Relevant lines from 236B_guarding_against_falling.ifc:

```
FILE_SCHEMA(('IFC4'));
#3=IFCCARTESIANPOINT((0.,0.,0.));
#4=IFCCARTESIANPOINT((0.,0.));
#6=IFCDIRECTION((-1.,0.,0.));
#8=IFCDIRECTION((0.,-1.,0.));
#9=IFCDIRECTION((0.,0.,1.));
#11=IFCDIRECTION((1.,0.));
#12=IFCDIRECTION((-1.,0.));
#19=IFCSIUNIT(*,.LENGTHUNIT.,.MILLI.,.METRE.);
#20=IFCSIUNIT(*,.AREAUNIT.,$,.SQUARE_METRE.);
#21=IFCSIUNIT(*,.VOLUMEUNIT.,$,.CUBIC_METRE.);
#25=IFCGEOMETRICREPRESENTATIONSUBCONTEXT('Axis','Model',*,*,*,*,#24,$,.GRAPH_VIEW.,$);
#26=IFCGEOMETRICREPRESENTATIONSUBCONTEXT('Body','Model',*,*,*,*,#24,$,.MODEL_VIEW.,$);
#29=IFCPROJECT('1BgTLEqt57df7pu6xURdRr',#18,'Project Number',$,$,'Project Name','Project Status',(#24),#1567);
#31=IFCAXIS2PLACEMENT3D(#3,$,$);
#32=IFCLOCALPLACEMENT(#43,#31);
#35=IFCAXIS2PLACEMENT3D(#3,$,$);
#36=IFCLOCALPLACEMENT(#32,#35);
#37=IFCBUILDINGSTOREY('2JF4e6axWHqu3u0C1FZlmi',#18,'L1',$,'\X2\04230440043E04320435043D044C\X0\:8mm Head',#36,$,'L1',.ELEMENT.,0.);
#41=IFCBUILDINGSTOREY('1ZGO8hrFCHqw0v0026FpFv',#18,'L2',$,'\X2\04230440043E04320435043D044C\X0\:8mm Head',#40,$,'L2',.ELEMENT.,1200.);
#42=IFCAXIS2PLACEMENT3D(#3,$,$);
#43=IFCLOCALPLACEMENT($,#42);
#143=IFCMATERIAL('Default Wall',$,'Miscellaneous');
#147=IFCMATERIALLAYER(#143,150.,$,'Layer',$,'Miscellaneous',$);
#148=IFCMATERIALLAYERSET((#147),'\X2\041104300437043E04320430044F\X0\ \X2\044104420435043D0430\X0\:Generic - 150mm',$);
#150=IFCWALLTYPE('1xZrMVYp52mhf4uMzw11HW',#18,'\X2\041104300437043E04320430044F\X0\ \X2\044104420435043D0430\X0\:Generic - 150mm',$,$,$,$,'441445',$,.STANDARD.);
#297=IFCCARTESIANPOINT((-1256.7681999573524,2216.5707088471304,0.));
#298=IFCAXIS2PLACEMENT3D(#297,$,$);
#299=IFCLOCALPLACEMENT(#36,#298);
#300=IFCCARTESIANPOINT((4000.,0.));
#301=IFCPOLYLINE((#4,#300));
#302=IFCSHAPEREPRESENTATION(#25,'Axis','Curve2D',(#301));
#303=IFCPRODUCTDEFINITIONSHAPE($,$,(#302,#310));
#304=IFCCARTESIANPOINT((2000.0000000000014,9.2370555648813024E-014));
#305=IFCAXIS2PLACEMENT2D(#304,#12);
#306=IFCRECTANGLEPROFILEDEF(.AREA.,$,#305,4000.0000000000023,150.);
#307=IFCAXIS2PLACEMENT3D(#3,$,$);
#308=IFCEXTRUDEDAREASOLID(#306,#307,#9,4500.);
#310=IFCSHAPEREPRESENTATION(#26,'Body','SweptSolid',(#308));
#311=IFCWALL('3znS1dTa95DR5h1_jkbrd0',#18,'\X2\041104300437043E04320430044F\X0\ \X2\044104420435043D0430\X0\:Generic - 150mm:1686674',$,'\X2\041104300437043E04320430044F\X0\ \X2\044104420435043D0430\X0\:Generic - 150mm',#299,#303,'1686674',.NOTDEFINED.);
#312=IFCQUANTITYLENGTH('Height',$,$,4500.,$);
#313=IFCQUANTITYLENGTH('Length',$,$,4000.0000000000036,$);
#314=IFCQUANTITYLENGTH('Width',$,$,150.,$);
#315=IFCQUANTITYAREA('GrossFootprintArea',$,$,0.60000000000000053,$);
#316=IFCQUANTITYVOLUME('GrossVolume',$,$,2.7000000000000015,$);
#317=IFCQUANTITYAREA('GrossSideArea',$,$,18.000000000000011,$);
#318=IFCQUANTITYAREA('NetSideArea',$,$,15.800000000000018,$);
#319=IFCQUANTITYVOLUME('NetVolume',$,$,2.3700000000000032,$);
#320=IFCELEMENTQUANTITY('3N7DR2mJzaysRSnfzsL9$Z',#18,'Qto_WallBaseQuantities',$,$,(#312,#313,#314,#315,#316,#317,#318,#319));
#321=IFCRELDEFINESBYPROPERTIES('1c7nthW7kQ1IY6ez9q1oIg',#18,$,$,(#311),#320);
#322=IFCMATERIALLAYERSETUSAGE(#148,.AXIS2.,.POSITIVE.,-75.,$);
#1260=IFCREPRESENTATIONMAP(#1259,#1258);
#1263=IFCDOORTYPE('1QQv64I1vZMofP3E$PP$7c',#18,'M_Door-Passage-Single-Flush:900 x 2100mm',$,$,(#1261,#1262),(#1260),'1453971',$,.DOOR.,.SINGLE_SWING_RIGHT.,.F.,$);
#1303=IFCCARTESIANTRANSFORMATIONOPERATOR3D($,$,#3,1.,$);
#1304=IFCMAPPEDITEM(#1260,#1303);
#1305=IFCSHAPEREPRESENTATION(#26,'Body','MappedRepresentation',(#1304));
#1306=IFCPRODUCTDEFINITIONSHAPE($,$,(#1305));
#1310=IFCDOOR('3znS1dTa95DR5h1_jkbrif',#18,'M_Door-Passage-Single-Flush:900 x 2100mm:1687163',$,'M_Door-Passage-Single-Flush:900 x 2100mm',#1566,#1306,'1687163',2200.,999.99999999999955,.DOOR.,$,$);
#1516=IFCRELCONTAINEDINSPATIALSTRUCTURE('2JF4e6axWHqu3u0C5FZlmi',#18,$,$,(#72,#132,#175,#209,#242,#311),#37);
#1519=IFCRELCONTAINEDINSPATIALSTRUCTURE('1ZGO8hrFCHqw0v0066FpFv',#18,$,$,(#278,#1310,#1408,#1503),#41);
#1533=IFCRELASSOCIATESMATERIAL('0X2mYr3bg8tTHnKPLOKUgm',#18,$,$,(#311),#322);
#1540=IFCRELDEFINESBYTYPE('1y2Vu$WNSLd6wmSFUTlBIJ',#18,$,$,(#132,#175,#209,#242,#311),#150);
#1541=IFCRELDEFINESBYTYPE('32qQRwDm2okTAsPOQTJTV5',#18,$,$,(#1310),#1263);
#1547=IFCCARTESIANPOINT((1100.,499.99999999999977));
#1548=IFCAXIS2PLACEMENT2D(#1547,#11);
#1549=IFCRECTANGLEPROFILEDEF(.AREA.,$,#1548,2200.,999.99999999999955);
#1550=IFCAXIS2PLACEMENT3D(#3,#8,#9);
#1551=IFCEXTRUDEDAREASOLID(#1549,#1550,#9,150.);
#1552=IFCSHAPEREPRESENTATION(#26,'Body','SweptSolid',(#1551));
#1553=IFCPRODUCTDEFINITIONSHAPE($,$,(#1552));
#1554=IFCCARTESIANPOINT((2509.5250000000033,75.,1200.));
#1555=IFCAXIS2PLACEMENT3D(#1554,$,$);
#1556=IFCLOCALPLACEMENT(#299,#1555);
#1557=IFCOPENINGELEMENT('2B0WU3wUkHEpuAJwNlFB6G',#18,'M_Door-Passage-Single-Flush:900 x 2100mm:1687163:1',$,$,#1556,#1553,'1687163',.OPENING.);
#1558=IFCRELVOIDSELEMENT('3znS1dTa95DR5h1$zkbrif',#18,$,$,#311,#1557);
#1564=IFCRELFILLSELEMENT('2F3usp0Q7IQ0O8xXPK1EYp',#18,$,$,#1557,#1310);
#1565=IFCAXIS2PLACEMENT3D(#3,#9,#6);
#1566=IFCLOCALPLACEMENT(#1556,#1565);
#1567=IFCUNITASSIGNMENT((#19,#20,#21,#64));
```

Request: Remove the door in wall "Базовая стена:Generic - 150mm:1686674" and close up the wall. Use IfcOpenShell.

```python
import ifcopenshell
import ifcopenshell.api.feature
import ifcopenshell.api.pset
import ifcopenshell.api.root
import ifcopenshell.geom
import ifcopenshell.util.element
import ifcopenshell.util.shape
import ifcopenshell.util.unit

model = ifcopenshell.open("236B_guarding_against_falling.ifc")
area_scale = ifcopenshell.util.unit.calculate_unit_scale(model, "AREAUNIT")
volume_scale = ifcopenshell.util.unit.calculate_unit_scale(model, "VOLUMEUNIT")
settings = ifcopenshell.geom.settings()


def volume(element):
    """Net volume in cubic metres, openings subtracted."""
    shape = ifcopenshell.geom.create_shape(settings, element)
    return ifcopenshell.util.shape.get_volume(shape.geometry)


door = model.by_id(1310)
opening = door.FillsVoids[0].RelatingOpeningElement
wall = opening.VoidsElements[0].RelatingBuildingElement
before = volume(wall)

ifcopenshell.api.root.remove_product(model, product=door)
ifcopenshell.api.feature.remove_feature(model, feature=opening)

after = volume(wall)
thickness = 0.15  # wall thickness in metres

# Update the wall's stored quantities.
qto = model.by_id(ifcopenshell.util.element.get_pset(wall, "Qto_WallBaseQuantities", should_inherit=False)["id"])
ifcopenshell.api.pset.edit_qto(model, qto=qto, properties={
    "NetSideArea": after / thickness / area_scale,
    "NetVolume": after / volume_scale,
})

print(f"wall volume {before:.3f} -> {after:.3f} m3")

model.write("236B_guarding_against_falling_v2.ifc")
```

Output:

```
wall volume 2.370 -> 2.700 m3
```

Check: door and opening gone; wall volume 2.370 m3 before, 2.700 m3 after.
